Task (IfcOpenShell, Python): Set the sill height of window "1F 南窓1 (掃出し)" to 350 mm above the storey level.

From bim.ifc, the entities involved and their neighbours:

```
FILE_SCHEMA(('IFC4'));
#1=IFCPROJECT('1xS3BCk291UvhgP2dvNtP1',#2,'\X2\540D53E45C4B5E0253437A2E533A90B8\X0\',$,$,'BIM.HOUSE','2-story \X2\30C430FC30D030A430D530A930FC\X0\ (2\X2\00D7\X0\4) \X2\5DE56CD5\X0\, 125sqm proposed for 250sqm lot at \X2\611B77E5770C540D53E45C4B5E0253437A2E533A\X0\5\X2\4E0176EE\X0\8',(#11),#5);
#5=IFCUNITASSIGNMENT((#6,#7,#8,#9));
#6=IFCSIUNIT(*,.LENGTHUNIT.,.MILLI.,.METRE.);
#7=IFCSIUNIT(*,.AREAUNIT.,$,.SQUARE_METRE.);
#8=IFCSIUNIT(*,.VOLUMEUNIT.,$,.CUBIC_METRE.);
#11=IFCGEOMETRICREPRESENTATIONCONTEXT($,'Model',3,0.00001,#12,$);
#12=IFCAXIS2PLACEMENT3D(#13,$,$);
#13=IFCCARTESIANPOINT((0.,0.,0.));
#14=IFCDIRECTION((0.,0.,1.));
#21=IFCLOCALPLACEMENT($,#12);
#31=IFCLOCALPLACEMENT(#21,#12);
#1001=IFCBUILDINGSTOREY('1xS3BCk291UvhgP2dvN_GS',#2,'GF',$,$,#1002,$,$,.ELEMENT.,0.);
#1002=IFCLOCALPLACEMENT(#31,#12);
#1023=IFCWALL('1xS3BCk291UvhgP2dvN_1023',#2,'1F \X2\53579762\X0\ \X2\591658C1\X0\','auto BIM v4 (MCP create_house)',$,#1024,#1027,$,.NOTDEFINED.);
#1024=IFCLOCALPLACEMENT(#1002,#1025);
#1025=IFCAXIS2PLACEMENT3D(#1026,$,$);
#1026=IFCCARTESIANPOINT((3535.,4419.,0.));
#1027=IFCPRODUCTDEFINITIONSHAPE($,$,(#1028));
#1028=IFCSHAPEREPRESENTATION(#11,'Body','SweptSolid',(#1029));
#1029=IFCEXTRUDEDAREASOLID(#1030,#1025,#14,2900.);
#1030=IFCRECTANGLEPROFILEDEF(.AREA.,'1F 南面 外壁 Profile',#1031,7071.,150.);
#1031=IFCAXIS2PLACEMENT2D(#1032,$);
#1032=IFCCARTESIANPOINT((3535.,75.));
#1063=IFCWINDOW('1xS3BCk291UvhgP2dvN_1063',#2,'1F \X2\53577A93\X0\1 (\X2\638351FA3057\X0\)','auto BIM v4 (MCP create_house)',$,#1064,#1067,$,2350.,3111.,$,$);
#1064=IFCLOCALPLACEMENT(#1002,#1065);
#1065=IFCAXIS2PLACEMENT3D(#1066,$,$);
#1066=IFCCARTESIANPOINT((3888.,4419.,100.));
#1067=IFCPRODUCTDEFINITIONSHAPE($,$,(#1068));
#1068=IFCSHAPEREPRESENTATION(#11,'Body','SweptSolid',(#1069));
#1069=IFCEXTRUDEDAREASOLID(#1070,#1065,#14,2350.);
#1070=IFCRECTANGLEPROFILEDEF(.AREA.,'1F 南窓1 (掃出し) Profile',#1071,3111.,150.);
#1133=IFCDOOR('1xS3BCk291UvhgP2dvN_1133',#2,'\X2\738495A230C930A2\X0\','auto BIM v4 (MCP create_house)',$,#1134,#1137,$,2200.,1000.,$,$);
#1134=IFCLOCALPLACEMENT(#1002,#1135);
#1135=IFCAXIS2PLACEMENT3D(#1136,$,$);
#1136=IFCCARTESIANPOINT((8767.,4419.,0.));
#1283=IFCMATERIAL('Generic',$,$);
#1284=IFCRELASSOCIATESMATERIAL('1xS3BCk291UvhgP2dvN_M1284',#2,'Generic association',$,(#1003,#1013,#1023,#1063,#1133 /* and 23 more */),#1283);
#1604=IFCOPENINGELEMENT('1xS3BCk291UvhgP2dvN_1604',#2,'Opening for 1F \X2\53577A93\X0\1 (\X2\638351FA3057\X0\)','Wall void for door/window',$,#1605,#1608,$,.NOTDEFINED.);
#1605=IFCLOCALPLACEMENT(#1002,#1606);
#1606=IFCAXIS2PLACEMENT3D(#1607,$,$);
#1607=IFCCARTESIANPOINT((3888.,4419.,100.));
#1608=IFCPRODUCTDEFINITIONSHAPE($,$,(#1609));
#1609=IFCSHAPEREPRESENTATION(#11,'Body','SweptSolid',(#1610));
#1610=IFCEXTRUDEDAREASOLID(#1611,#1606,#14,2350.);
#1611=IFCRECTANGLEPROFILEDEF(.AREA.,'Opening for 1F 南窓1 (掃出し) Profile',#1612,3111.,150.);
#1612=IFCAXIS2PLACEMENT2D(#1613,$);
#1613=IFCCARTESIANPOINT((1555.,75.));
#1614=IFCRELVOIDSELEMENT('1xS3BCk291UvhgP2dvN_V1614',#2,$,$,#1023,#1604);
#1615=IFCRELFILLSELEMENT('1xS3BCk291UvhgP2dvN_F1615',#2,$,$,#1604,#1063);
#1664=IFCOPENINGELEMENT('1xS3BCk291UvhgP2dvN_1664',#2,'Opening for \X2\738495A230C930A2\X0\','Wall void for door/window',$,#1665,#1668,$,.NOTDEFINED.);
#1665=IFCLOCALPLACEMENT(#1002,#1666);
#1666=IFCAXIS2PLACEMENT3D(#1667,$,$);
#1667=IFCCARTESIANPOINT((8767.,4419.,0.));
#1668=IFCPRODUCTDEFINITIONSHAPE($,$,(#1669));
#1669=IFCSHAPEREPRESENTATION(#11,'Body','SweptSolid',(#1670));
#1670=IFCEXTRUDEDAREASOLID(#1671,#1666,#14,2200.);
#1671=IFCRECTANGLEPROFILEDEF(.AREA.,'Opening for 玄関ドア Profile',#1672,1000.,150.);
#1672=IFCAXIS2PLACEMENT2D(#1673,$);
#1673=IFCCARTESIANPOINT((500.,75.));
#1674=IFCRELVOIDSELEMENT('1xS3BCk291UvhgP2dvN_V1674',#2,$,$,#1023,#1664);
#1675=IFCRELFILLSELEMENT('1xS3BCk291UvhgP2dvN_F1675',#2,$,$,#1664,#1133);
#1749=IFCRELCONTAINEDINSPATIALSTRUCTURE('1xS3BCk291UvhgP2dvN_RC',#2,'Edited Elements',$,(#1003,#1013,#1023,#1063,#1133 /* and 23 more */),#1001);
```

```python
import numpy as np
import ifcopenshell
import ifcopenshell.api.geometry
import ifcopenshell.geom
import ifcopenshell.util.element
import ifcopenshell.util.placement
import ifcopenshell.util.shape
import ifcopenshell.util.unit

model = ifcopenshell.open("bim.ifc")
unit_scale = ifcopenshell.util.unit.calculate_unit_scale(model)

window = model.by_guid("1xS3BCk291UvhgP2dvN_1063")
opening = window.FillsVoids[0].RelatingOpeningElement
storey = ifcopenshell.util.element.get_container(window, ifc_class="IfcBuildingStorey")
level = ifcopenshell.util.placement.get_local_placement(storey.ObjectPlacement)[2, 3]

# The opening's origin need not be at the sill, so measure its lowest point.
shape = ifcopenshell.geom.create_shape(ifcopenshell.geom.settings(), opening)
bottom = ifcopenshell.util.shape.get_shape_bottom_elevation(shape, shape.geometry) / unit_scale
dz = level + 0.35 / unit_scale - bottom

shift = np.array([0.0, 0.0, dz])
# The window is not placed relative to its opening, so move both.
for product in (opening, window):
    matrix = ifcopenshell.util.placement.get_local_placement(product.ObjectPlacement)
    matrix[:3, 3] += shift
    ifcopenshell.api.geometry.edit_object_placement(model, product=product, matrix=matrix, is_si=False)

print(f"moved by {dz * unit_scale:+.3f} m")

model.write("bim_updated.ifc")
```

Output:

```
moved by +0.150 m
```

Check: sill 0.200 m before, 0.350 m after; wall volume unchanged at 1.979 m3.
